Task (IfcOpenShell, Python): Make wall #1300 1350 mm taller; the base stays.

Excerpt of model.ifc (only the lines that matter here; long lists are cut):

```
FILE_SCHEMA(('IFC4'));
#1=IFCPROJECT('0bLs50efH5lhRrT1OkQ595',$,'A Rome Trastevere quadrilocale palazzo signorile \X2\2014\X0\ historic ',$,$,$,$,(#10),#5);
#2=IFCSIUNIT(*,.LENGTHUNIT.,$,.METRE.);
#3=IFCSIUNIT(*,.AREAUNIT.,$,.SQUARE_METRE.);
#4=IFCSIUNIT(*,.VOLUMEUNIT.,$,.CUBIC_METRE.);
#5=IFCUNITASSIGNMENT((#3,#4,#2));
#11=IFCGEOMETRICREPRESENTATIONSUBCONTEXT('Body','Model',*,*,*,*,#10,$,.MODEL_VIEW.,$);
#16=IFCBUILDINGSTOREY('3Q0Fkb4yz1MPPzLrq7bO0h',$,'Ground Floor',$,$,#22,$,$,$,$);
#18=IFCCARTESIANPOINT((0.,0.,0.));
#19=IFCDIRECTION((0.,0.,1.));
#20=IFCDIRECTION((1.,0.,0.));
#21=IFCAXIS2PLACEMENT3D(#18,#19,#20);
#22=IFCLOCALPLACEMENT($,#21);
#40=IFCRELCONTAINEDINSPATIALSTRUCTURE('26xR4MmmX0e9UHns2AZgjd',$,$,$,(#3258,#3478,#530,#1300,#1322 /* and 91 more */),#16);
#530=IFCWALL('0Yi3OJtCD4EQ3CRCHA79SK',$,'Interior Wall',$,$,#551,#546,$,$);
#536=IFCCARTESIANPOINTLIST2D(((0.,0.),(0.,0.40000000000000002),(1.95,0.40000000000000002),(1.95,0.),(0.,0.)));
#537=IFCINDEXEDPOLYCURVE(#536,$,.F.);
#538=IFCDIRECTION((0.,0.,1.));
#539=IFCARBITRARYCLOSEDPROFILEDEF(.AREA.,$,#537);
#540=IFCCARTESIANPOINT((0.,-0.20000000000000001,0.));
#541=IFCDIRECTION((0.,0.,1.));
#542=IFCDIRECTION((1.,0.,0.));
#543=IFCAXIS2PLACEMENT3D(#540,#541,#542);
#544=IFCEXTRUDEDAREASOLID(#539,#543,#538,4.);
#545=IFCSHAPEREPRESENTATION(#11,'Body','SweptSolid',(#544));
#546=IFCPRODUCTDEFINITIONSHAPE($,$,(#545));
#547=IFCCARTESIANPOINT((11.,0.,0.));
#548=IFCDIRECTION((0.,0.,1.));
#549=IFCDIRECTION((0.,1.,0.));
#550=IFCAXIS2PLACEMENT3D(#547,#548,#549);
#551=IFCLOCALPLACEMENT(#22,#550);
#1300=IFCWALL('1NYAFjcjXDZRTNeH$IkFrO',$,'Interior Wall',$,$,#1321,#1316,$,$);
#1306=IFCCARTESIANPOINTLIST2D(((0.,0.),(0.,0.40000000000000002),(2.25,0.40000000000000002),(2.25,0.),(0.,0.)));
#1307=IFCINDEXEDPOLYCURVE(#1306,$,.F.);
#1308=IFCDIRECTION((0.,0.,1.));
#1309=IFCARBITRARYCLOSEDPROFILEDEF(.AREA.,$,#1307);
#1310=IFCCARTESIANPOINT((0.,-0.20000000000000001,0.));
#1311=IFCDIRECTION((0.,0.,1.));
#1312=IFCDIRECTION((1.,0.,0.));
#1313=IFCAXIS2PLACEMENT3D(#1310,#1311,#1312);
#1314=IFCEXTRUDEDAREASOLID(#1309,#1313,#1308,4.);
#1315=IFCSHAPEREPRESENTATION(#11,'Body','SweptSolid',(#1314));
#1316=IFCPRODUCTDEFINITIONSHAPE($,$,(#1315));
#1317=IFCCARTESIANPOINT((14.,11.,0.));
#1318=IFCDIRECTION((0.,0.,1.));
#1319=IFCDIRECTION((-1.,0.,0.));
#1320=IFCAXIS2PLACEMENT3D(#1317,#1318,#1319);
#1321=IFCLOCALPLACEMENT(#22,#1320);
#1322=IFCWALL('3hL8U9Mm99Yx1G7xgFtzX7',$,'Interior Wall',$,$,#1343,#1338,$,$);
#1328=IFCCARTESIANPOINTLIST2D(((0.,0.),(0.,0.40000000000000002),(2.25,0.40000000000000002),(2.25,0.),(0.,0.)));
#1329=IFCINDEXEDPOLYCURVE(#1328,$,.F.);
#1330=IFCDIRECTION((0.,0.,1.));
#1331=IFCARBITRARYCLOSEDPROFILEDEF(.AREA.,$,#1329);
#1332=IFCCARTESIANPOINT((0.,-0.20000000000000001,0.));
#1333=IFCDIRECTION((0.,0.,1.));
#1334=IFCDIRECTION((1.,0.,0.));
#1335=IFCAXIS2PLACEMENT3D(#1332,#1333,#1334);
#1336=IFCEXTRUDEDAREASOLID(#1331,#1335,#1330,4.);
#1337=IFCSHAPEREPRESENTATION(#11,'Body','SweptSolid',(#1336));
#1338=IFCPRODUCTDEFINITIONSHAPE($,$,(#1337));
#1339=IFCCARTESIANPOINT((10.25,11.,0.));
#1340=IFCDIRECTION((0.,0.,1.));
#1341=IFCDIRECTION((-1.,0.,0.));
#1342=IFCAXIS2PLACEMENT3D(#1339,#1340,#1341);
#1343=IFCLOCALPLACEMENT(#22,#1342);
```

```python
import ifcopenshell
import ifcopenshell.geom
import ifcopenshell.util.representation
import ifcopenshell.util.shape
import ifcopenshell.util.unit

model = ifcopenshell.open("model.ifc")
unit_scale = ifcopenshell.util.unit.calculate_unit_scale(model)
settings = ifcopenshell.geom.settings()


def volume(element):
    """Net volume in cubic metres, openings subtracted."""
    shape = ifcopenshell.geom.create_shape(settings, element)
    return ifcopenshell.util.shape.get_volume(shape.geometry)


wall = model.by_guid("1NYAFjcjXDZRTNeH$IkFrO")
before = volume(wall)

body = ifcopenshell.util.representation.get_representation(wall, "Model", "Body")
solid = body.Items[0]
old_height = solid.Depth
solid.Depth += 1.35 / unit_scale
after = volume(wall)

print(f"height {old_height:g} -> {solid.Depth:g}, volume {before:.3f} -> {after:.3f} m3")

model.write("model-out.ifc")
```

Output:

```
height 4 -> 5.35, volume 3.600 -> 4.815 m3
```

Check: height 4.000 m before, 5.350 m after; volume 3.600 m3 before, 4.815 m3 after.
